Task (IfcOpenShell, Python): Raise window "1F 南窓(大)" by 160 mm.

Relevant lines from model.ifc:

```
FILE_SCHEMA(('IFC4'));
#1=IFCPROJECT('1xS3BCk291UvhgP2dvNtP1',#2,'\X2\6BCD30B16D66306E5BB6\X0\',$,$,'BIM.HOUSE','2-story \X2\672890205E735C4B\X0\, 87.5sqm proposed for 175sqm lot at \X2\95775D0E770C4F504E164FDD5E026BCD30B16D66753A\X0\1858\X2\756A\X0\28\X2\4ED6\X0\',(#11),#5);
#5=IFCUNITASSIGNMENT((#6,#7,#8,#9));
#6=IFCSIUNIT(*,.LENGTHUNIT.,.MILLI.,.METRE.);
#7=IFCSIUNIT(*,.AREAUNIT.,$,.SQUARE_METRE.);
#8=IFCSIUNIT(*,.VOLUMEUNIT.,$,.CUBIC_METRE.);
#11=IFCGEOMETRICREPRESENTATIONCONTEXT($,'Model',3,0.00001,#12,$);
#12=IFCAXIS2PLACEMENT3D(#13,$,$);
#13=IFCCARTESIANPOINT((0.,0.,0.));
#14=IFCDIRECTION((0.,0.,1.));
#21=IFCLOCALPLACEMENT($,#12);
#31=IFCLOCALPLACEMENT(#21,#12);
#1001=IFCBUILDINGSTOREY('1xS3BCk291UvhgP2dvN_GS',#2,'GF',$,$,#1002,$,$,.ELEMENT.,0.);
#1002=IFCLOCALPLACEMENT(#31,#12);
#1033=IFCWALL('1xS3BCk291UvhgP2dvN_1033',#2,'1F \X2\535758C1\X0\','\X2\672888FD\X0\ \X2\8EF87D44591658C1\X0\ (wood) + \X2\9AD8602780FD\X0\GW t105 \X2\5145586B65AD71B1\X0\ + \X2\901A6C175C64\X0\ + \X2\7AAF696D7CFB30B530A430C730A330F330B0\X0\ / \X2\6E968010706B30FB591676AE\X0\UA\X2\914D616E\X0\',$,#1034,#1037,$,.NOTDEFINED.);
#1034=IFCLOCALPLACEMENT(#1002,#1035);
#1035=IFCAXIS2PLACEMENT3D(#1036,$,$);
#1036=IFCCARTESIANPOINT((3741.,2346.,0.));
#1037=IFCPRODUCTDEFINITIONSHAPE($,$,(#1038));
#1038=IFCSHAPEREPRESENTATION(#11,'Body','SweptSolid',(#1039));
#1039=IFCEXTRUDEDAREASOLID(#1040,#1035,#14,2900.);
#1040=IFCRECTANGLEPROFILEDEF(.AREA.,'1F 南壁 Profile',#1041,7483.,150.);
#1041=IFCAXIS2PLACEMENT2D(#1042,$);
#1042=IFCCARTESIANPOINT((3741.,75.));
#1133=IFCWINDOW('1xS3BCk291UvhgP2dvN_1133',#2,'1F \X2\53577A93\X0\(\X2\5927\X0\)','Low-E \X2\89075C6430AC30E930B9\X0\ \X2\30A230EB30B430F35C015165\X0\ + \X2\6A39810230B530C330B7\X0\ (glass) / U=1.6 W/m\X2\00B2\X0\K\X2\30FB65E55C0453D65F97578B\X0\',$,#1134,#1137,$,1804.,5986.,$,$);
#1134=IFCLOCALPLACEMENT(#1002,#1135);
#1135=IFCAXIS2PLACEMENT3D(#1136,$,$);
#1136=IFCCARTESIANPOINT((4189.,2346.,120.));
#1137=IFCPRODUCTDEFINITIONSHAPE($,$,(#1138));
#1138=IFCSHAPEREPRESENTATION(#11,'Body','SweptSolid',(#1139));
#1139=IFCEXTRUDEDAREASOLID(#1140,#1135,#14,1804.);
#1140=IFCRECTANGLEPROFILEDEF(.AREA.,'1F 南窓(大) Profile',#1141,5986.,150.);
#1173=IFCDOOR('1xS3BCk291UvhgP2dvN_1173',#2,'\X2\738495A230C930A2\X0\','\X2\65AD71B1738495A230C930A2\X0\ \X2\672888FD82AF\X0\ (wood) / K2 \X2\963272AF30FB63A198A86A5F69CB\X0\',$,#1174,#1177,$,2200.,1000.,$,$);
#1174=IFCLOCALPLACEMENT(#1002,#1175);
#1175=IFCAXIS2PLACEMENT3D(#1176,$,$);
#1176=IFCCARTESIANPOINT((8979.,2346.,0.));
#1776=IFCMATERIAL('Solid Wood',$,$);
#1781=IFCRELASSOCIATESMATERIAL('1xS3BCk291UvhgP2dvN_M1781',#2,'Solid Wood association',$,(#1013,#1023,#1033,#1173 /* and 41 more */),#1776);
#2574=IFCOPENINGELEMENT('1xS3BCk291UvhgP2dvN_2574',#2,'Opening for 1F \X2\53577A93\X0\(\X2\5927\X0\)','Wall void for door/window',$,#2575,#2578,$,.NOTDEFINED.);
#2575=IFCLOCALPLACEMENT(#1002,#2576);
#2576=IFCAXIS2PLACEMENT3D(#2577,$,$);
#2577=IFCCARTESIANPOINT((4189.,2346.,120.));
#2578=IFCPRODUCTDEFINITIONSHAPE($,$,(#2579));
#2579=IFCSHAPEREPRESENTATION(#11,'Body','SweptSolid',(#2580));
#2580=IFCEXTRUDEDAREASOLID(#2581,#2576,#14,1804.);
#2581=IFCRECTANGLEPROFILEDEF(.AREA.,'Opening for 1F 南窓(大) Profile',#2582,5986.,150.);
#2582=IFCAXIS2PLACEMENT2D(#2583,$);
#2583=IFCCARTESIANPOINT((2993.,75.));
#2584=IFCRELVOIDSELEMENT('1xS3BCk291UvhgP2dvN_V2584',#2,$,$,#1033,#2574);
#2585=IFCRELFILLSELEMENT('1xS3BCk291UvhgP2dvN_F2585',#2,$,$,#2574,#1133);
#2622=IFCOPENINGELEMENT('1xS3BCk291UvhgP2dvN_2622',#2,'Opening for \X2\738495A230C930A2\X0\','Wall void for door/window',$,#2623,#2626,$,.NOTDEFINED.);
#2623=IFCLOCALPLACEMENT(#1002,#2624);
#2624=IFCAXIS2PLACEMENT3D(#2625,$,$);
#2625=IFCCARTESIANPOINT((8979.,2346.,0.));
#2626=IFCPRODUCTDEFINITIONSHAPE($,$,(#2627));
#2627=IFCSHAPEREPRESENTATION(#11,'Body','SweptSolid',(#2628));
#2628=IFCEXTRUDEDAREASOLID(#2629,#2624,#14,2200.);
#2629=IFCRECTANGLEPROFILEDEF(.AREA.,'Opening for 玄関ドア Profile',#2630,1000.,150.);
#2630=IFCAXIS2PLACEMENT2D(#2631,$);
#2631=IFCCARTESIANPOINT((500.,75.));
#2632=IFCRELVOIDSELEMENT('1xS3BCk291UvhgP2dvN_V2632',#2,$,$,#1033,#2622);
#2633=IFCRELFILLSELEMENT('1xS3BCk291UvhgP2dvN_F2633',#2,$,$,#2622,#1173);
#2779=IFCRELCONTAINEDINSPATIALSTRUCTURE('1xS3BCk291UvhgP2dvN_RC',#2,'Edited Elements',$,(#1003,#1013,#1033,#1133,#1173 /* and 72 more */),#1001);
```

```python
import numpy as np
import ifcopenshell
import ifcopenshell.api.geometry
import ifcopenshell.util.placement
import ifcopenshell.util.unit

model = ifcopenshell.open("model.ifc")
unit_scale = ifcopenshell.util.unit.calculate_unit_scale(model)

window = model.by_guid("1xS3BCk291UvhgP2dvN_1133")
opening = window.FillsVoids[0].RelatingOpeningElement
dz = 0.16 / unit_scale

shift = np.array([0.0, 0.0, dz])
# The window is not placed relative to its opening, so move both.
for product in (opening, window):
    matrix = ifcopenshell.util.placement.get_local_placement(product.ObjectPlacement)
    matrix[:3, 3] += shift
    ifcopenshell.api.geometry.edit_object_placement(model, product=product, matrix=matrix, is_si=False)

print(f"moved by {dz * unit_scale:+.3f} m")

model.write("model_updated.ifc")
```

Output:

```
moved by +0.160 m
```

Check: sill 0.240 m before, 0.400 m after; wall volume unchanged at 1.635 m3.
